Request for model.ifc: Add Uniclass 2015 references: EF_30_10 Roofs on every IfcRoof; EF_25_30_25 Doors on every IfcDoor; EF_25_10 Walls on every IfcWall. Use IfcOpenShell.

First a look at what the model holds.

```python
import ifcopenshell

model = ifcopenshell.open("model.ifc")
print(model.schema)
print("classifications:", [c.Name for c in model.by_type("IfcClassification")])
for ifc_class in ("IfcDoor", "IfcRoof", "IfcStair", "IfcWall", "IfcWindow"):
    print(ifc_class, len(model.by_type(ifc_class)))
```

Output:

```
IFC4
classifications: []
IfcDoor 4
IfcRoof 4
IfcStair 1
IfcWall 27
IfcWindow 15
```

```python
import ifcopenshell
import ifcopenshell.api.classification

model = ifcopenshell.open("model.ifc")

system = ifcopenshell.api.classification.add_classification(model, classification="Uniclass 2015")

codes = {
    "IfcRoof": ("EF_30_10", "Roofs"),
    "IfcDoor": ("EF_25_30_25", "Doors"),
    "IfcWall": ("EF_25_10", "Walls"),
}
for ifc_class, (code, name) in codes.items():
    products = model.by_type(ifc_class)
    ifcopenshell.api.classification.add_reference(
        model, products=products, classification=system, identification=code, name=name
    )
    print(code, len(products))

model.write("model_rev.ifc")
```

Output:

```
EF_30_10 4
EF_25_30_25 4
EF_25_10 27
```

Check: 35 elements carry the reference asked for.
